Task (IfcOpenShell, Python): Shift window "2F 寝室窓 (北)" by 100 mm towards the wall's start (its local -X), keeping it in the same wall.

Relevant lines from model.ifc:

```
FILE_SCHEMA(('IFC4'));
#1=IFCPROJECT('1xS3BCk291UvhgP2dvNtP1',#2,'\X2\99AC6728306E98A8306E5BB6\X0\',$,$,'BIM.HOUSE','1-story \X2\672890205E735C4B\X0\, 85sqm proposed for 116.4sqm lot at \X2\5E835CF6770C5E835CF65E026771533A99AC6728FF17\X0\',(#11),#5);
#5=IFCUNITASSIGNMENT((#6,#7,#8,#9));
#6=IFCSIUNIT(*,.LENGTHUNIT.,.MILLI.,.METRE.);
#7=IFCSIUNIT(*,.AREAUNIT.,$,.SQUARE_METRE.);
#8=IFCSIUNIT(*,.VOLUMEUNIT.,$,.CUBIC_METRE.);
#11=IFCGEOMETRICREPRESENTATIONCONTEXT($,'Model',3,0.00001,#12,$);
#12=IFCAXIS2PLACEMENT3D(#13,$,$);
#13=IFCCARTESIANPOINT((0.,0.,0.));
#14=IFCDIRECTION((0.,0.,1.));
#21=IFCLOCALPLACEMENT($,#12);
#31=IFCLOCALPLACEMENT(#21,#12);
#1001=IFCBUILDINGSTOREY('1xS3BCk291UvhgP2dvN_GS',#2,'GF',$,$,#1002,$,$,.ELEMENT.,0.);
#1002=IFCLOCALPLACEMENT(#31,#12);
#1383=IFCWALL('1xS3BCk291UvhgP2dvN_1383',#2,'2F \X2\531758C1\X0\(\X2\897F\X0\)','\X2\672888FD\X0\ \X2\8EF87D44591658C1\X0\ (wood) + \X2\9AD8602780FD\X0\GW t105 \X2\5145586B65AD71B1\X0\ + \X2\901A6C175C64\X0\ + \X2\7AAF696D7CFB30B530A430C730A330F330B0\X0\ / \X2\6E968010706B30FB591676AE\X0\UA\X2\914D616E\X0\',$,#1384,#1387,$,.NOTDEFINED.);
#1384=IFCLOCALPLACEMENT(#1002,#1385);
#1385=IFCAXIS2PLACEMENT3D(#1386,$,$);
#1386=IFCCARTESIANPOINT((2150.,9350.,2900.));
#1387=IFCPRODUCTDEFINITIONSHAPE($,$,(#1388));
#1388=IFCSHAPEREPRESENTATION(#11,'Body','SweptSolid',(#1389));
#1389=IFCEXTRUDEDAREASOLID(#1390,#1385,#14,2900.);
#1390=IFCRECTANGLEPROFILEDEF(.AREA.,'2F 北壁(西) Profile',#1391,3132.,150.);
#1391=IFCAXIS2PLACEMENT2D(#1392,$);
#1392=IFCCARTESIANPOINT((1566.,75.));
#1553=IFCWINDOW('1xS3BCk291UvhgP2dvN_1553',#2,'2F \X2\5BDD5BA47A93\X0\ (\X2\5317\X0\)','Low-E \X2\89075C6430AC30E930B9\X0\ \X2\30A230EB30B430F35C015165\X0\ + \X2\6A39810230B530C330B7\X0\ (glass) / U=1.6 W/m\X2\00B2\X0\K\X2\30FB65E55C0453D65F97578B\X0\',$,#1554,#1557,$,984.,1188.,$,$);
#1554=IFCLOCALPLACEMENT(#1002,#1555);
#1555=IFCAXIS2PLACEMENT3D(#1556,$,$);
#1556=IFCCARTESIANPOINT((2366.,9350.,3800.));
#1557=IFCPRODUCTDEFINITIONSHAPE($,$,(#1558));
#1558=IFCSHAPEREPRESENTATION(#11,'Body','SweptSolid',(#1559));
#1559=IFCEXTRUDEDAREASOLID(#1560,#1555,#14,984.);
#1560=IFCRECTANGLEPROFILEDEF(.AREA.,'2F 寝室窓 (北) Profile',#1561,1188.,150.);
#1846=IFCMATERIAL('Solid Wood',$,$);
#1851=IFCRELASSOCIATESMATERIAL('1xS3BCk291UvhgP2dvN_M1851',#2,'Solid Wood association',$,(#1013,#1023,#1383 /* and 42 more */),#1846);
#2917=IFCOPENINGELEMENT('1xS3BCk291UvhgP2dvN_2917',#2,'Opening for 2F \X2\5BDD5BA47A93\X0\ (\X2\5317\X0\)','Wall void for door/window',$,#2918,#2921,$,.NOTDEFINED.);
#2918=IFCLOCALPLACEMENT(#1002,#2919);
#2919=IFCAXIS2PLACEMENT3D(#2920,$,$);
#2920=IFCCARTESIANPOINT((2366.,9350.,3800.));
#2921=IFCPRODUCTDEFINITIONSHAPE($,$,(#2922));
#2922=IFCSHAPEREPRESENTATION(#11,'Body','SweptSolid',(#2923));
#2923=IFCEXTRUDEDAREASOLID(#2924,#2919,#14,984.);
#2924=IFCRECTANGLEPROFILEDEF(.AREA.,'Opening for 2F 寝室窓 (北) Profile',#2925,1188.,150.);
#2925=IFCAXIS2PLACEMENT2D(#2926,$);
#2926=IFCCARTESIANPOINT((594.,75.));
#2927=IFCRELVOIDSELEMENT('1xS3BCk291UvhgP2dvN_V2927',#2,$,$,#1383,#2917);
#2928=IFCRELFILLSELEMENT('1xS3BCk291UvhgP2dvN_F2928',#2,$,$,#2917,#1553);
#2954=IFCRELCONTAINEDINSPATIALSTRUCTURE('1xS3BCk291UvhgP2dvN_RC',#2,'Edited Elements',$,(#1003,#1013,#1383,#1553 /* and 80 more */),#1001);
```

```python
import ifcopenshell
import ifcopenshell.api.geometry
import ifcopenshell.util.placement

model = ifcopenshell.open("model.ifc")

window = model.by_id(1553)
opening = window.FillsVoids[0].RelatingOpeningElement
wall = opening.VoidsElements[0].RelatingBuildingElement

wall_matrix = ifcopenshell.util.placement.get_local_placement(wall.ObjectPlacement)
shift = wall_matrix[:3, 0] * -100.0
before = ifcopenshell.util.placement.get_local_placement(window.ObjectPlacement)[:3, 3].copy()

# The window is not placed relative to its opening, so move both.
for product in (opening, window):
    matrix = ifcopenshell.util.placement.get_local_placement(product.ObjectPlacement)
    matrix[:3, 3] += shift
    ifcopenshell.api.geometry.edit_object_placement(model, product=product, matrix=matrix, is_si=False)

after = ifcopenshell.util.placement.get_local_placement(window.ObjectPlacement)[:3, 3]
print("window moved by", (after - before).round(3) + 0.0)

model.write("model_rev.ifc")
```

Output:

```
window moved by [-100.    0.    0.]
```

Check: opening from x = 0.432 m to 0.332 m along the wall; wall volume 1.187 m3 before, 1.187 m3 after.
